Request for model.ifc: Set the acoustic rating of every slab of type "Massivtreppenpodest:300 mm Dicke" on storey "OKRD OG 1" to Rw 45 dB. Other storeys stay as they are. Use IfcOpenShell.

First a look at what the model holds.

```python
import ifcopenshell
import ifcopenshell.util.element

model = ifcopenshell.open("model.ifc")
print(model.schema)
storey = next(s for s in model.by_type("IfcBuildingStorey") if s.Name == "OKRD OG 1")
slabs = [e for e in ifcopenshell.util.element.get_decomposition(storey) if e.is_a("IfcSlab")]
seen = {}
for e in slabs:
    element_type = ifcopenshell.util.element.get_type(e)
    key = (element_type.Name if element_type != e and element_type else None, ifcopenshell.util.element.get_pset(e, "Pset_SlabCommon", "AcousticRating"))
    seen[key] = seen.get(key, 0) + 1
for (name, value), count in sorted(seen.items(), key=str):
    print(count, "x", name, "|", value)
```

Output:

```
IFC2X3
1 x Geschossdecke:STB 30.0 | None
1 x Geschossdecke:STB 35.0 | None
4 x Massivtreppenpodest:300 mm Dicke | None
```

```python
import ifcopenshell
import ifcopenshell.api.pset
import ifcopenshell.util.element

model = ifcopenshell.open("model.ifc")

storey = next(s for s in model.by_type("IfcBuildingStorey") if s.Name == "OKRD OG 1")
slabs = [e for e in ifcopenshell.util.element.get_decomposition(storey) if e.is_a("IfcSlab")]

count = 0
for e in slabs:
    element_type = ifcopenshell.util.element.get_type(e)
    if element_type in (None, e) or element_type.Name != "Massivtreppenpodest:300 mm Dicke":
        continue
    found = ifcopenshell.util.element.get_pset(e, "Pset_SlabCommon", should_inherit=False)
    if found:
        pset = model.by_id(found["id"])
        if len(ifcopenshell.util.element.get_elements_by_pset(pset)) > 1:
            pset = ifcopenshell.api.pset.unshare_pset(model, products=[e], pset=pset)[0]
    else:
        pset = ifcopenshell.api.pset.add_pset(model, product=e, name="Pset_SlabCommon")
    ifcopenshell.api.pset.edit_pset(model, pset=pset, properties={"AcousticRating": "Rw 45 dB"})
    count += 1

print(count, "slabs updated")

model.write("model_updated.ifc")
```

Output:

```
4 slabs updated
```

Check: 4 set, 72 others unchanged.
